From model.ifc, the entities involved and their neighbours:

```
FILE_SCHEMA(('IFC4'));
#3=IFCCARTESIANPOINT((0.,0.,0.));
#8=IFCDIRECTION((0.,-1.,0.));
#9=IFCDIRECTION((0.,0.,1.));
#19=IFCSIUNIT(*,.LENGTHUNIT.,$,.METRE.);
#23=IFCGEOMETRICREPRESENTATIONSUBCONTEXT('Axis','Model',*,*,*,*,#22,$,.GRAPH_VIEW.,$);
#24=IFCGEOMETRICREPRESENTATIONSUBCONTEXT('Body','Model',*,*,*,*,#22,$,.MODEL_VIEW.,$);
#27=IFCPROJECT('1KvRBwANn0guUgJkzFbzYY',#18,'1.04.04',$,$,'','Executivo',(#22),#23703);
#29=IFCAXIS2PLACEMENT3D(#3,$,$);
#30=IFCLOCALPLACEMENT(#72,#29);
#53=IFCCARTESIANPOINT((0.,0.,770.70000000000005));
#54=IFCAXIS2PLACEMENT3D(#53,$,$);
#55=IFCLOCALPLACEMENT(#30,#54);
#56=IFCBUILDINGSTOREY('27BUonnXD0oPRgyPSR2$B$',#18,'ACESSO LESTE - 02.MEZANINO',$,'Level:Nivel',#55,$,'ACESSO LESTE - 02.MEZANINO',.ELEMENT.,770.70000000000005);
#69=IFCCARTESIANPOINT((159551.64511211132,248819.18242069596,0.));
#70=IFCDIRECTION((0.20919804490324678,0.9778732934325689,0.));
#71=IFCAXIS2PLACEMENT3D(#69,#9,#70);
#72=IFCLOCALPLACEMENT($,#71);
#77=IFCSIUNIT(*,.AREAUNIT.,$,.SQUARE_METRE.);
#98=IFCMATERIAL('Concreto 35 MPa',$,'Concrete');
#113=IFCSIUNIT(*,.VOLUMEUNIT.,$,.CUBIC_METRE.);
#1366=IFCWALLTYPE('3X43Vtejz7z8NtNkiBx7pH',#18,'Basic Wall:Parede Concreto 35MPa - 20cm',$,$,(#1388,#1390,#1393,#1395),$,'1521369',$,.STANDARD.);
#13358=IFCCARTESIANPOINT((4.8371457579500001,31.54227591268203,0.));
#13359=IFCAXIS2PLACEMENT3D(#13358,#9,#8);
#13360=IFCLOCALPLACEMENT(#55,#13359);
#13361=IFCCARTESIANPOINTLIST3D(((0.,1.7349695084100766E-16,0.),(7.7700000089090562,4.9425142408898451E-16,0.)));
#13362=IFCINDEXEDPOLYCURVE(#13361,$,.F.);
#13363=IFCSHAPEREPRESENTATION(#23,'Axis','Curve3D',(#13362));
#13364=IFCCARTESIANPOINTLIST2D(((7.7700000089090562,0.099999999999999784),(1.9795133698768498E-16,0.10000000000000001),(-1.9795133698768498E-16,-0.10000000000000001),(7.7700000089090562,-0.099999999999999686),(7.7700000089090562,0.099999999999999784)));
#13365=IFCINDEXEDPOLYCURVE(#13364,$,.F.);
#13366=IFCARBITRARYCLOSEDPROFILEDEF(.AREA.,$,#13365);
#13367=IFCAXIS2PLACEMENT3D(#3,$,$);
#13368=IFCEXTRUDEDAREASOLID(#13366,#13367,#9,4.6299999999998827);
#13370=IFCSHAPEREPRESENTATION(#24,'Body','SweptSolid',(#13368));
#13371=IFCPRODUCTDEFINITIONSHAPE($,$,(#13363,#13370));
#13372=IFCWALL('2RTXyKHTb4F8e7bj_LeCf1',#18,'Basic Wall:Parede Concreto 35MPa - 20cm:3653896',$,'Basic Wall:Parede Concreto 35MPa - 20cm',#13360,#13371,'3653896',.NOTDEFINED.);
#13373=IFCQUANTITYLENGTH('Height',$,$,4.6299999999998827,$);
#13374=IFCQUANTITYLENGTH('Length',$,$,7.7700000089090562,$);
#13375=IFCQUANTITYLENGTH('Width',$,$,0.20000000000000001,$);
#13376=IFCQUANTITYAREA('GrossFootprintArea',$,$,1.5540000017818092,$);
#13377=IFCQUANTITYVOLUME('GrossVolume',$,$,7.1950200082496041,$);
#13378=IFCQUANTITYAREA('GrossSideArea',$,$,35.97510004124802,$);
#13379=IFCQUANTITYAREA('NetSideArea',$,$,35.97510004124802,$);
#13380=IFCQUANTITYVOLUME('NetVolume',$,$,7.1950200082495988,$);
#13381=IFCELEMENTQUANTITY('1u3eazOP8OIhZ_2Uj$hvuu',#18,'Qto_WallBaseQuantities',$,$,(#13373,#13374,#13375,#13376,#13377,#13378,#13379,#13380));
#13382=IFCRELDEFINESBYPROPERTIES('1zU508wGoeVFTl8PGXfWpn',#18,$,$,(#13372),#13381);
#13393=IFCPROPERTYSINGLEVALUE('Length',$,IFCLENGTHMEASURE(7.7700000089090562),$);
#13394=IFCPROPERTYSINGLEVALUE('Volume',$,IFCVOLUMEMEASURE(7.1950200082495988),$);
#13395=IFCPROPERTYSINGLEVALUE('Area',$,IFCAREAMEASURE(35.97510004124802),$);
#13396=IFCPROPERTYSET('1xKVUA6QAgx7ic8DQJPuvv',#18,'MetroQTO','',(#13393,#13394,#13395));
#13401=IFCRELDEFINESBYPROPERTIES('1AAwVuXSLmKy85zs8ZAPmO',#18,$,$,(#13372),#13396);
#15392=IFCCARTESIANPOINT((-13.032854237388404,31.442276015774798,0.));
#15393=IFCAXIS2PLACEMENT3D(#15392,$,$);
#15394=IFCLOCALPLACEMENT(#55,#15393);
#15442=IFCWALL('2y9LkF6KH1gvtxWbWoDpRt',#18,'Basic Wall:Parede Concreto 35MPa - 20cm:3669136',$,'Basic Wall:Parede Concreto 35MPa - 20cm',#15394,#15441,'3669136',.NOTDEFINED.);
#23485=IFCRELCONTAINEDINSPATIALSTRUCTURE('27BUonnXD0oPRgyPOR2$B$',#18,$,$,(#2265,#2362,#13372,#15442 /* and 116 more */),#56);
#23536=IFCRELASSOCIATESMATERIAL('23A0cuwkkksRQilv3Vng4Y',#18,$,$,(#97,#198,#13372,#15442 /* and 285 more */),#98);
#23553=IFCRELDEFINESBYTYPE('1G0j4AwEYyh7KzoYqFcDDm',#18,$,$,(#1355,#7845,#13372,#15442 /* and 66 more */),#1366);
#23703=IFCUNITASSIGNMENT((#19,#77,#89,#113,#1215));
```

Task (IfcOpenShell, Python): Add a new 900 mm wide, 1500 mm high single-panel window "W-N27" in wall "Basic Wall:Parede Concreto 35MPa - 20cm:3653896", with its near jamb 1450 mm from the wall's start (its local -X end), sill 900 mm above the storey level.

```python
import numpy as np
import ifcopenshell
import ifcopenshell.api.feature
import ifcopenshell.api.geometry
import ifcopenshell.api.pset
import ifcopenshell.api.root
import ifcopenshell.api.spatial
import ifcopenshell.geom
import ifcopenshell.util.element
import ifcopenshell.util.placement
import ifcopenshell.util.representation
import ifcopenshell.util.shape
import ifcopenshell.util.unit

model = ifcopenshell.open("model.ifc")
unit_scale = ifcopenshell.util.unit.calculate_unit_scale(model)
area_scale = ifcopenshell.util.unit.calculate_unit_scale(model, "AREAUNIT")
volume_scale = ifcopenshell.util.unit.calculate_unit_scale(model, "VOLUMEUNIT")
settings = ifcopenshell.geom.settings()


def volume(element):
    """Net volume in cubic metres, openings subtracted."""
    shape = ifcopenshell.geom.create_shape(settings, element)
    return ifcopenshell.util.shape.get_volume(shape.geometry)


wall = model.by_id(13372)
storey = ifcopenshell.util.element.get_container(wall, ifc_class="IfcBuildingStorey")
context = ifcopenshell.util.representation.get_context(model, "Model", "Body", "MODEL_VIEW")
before = volume(wall)

width, height, from_end, sill = 0.9, 1.5, 1.45, 0.9  # metres

# The wall runs along its own X axis, and the end named is its -X end.
wall_shape = ifcopenshell.geom.create_shape(settings, wall)
x, y, z = ifcopenshell.util.shape.get_vertices(wall_shape.geometry).T
start = x.min() + from_end
face, thickness = float(y.min()), float(y.max() - y.min())
wall_matrix = ifcopenshell.util.placement.get_local_placement(wall.ObjectPlacement)
level = ifcopenshell.util.placement.get_local_placement(storey.ObjectPlacement)[2, 3]


def in_wall(x, y):
    """Placement at x, y metres in the wall's axes, at sill height."""
    matrix = wall_matrix.copy()
    matrix[:, 3] = wall_matrix @ np.array([x / unit_scale, y / unit_scale, 0.0, 1.0])
    matrix[2, 3] = level + sill / unit_scale
    return matrix


# Opening: a box that overshoots both wall faces by 50 mm.
opening = ifcopenshell.api.root.create_entity(model, ifc_class="IfcOpeningElement", predefined_type="OPENING")
box = ifcopenshell.api.geometry.add_wall_representation(
    model, context=context, length=width, height=height, thickness=thickness + 0.1
)
ifcopenshell.api.geometry.assign_representation(model, product=opening, representation=box)
ifcopenshell.api.geometry.edit_object_placement(model, product=opening, matrix=in_wall(start, face - 0.05), is_si=False)
ifcopenshell.api.feature.add_feature(model, feature=opening, element=wall)

window = ifcopenshell.api.root.create_entity(model, ifc_class="IfcWindow", name="W-N27", predefined_type="WINDOW")
window.OverallWidth, window.OverallHeight = width / unit_scale, height / unit_scale
window.PartitioningType = "SINGLE_PANEL"
body = ifcopenshell.api.geometry.add_window_representation(
    model,
    context=context,
    overall_width=window.OverallWidth,
    overall_height=window.OverallHeight,
    partition_type="SINGLE_PANEL",
)
ifcopenshell.api.geometry.assign_representation(model, product=window, representation=body)
ifcopenshell.api.spatial.assign_container(model, products=[window], relating_structure=storey)
ifcopenshell.api.feature.add_filling(model, opening=opening, element=window)

# Centre the window in the wall's thickness.
ifcopenshell.api.geometry.edit_object_placement(model, product=window, matrix=in_wall(start, face), is_si=False)
window_shape = ifcopenshell.geom.create_shape(settings, window)
depth = ifcopenshell.util.shape.get_vertices(window_shape.geometry)[:, 1]
offset = face + thickness / 2 - (depth.min() + depth.max()) / 2
ifcopenshell.api.geometry.edit_object_placement(model, product=window, matrix=in_wall(start, offset), is_si=False)

after = volume(wall)

# Update the wall's stored quantities.
qto = model.by_id(ifcopenshell.util.element.get_pset(wall, "Qto_WallBaseQuantities", should_inherit=False)["id"])
ifcopenshell.api.pset.edit_qto(model, qto=qto, properties={
    "NetSideArea": after / thickness / area_scale,
    "NetVolume": after / volume_scale,
})
pset = model.by_id(ifcopenshell.util.element.get_pset(wall, "MetroQTO", should_inherit=False)["id"])
ifcopenshell.api.pset.edit_pset(model, pset=pset, properties={
    "Volume": model.create_entity("IfcVolumeMeasure", after / volume_scale),
    "Area": model.create_entity("IfcAreaMeasure", after / thickness / area_scale),
})

print(f"wall volume {before:.3f} -> {after:.3f} m3")

model.write("model_v2.ifc")
```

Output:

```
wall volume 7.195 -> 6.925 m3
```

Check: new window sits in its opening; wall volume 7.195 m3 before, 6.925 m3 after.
